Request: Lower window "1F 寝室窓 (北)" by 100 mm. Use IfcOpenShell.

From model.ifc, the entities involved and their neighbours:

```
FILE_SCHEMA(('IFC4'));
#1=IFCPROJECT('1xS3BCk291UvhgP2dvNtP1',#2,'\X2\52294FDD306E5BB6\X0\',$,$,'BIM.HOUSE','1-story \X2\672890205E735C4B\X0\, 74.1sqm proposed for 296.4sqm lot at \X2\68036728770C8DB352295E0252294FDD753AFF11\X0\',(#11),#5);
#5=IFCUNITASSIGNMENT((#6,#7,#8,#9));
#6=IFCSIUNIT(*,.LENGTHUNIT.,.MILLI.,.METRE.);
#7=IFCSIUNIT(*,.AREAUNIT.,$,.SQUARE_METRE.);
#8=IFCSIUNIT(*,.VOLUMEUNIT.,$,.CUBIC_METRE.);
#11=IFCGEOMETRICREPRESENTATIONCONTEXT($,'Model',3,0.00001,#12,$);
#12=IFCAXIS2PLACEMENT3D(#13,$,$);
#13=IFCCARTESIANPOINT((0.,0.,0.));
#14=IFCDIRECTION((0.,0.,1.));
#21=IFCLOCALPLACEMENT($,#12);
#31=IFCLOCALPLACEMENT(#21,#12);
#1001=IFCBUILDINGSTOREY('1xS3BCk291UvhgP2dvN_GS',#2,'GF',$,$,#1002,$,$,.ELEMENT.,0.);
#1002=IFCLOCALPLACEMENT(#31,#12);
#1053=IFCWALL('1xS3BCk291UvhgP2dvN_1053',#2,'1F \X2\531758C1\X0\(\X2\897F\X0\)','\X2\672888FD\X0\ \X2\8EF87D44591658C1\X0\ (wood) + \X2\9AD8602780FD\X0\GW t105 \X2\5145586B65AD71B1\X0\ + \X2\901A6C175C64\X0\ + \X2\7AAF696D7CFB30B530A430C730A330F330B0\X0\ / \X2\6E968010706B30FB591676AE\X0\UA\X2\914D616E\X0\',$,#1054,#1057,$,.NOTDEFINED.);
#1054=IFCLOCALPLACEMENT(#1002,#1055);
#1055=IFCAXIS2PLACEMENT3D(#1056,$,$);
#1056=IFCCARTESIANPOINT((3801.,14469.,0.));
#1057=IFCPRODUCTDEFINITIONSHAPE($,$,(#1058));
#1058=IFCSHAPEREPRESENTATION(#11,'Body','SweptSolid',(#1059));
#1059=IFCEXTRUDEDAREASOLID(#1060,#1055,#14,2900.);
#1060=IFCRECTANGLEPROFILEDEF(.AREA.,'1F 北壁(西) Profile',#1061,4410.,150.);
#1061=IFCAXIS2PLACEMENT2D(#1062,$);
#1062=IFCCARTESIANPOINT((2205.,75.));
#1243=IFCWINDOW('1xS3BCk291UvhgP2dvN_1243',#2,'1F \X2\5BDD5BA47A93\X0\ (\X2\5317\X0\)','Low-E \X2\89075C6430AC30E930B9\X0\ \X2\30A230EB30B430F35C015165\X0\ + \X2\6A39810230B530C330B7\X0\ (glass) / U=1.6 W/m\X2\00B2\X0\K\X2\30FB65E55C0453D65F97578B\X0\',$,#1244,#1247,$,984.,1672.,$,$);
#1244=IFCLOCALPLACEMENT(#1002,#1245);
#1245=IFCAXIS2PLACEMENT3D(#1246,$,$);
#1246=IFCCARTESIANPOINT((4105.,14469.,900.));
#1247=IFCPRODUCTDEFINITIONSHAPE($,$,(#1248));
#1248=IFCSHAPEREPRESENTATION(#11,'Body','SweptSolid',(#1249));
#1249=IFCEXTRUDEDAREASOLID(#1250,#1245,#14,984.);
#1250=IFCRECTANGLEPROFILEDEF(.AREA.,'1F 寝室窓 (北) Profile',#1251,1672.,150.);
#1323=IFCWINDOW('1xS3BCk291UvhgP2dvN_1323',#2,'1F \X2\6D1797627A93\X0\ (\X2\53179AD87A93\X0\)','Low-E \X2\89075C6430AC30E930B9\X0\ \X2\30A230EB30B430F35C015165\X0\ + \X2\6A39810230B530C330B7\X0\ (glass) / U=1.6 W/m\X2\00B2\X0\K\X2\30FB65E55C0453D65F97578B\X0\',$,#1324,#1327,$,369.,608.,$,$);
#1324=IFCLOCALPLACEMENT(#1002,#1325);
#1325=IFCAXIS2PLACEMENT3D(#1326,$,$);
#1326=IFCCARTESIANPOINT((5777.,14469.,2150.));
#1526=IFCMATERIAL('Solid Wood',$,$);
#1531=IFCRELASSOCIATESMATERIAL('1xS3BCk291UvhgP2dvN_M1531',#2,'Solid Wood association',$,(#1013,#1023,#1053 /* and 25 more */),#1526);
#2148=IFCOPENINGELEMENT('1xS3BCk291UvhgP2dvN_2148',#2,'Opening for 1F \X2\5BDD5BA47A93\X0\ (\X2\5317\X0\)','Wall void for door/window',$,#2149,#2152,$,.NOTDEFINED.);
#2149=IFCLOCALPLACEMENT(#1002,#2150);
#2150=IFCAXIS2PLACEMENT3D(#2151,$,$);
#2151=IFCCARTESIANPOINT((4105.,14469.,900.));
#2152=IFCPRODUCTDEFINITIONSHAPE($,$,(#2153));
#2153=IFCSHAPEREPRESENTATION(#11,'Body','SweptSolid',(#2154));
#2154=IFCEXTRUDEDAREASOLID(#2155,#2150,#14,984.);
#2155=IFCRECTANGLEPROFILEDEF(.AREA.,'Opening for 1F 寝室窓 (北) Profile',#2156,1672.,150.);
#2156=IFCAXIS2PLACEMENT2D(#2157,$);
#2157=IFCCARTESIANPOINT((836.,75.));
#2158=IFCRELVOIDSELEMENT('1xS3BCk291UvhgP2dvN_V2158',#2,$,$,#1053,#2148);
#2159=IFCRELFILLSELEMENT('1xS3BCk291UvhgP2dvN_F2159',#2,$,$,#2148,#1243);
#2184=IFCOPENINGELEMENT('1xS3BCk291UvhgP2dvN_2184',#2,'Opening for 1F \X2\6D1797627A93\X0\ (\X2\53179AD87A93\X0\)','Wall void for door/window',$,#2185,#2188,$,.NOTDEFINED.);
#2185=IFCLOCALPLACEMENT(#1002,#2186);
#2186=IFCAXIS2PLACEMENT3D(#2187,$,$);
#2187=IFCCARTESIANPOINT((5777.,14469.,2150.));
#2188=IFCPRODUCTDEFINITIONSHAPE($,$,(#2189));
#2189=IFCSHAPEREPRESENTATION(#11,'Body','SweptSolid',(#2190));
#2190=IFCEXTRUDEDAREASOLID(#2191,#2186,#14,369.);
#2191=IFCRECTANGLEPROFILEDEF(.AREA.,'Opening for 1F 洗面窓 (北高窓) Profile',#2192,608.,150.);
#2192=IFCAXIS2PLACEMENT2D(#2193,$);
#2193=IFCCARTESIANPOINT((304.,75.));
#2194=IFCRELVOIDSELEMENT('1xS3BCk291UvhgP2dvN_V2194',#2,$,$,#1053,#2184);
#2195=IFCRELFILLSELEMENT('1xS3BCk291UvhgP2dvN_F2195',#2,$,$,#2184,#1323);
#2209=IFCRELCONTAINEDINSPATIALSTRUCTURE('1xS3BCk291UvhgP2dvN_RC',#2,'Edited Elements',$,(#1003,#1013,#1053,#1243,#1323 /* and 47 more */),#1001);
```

```python
import numpy as np
import ifcopenshell
import ifcopenshell.api.geometry
import ifcopenshell.util.placement
import ifcopenshell.util.unit

model = ifcopenshell.open("model.ifc")
unit_scale = ifcopenshell.util.unit.calculate_unit_scale(model)

window = model.by_guid("1xS3BCk291UvhgP2dvN_1243")
opening = window.FillsVoids[0].RelatingOpeningElement
dz = -100.0

shift = np.array([0.0, 0.0, dz])
# The window is not placed relative to its opening, so move both.
for product in (opening, window):
    matrix = ifcopenshell.util.placement.get_local_placement(product.ObjectPlacement)
    matrix[:3, 3] += shift
    ifcopenshell.api.geometry.edit_object_placement(model, product=product, matrix=matrix, is_si=False)

print(f"moved by {dz * unit_scale:+.3f} m")

model.write("model_v2.ifc")
```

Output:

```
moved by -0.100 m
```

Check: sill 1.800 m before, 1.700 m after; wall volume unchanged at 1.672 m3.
